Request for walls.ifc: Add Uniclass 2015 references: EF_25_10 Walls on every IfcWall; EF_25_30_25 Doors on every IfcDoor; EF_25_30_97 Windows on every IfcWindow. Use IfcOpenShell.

First a look at what the model holds.

```python
import ifcopenshell

model = ifcopenshell.open("walls.ifc")
print(model.schema)
print("classifications:", [c.Name for c in model.by_type("IfcClassification")])
for ifc_class in ("IfcDoor", "IfcRoof", "IfcStair", "IfcWall", "IfcWindow"):
    print(ifc_class, len(model.by_type(ifc_class)))
```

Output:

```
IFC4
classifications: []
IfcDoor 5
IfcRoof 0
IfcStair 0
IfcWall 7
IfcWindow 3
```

```python
import ifcopenshell
import ifcopenshell.api.classification

model = ifcopenshell.open("walls.ifc")

system = ifcopenshell.api.classification.add_classification(model, classification="Uniclass 2015")

codes = {
    "IfcWall": ("EF_25_10", "Walls"),
    "IfcDoor": ("EF_25_30_25", "Doors"),
    "IfcWindow": ("EF_25_30_97", "Windows"),
}
for ifc_class, (code, name) in codes.items():
    products = model.by_type(ifc_class)
    ifcopenshell.api.classification.add_reference(
        model, products=products, classification=system, identification=code, name=name
    )
    print(code, len(products))

model.write("walls_v2.ifc")
```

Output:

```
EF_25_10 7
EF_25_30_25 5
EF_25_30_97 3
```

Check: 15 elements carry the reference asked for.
